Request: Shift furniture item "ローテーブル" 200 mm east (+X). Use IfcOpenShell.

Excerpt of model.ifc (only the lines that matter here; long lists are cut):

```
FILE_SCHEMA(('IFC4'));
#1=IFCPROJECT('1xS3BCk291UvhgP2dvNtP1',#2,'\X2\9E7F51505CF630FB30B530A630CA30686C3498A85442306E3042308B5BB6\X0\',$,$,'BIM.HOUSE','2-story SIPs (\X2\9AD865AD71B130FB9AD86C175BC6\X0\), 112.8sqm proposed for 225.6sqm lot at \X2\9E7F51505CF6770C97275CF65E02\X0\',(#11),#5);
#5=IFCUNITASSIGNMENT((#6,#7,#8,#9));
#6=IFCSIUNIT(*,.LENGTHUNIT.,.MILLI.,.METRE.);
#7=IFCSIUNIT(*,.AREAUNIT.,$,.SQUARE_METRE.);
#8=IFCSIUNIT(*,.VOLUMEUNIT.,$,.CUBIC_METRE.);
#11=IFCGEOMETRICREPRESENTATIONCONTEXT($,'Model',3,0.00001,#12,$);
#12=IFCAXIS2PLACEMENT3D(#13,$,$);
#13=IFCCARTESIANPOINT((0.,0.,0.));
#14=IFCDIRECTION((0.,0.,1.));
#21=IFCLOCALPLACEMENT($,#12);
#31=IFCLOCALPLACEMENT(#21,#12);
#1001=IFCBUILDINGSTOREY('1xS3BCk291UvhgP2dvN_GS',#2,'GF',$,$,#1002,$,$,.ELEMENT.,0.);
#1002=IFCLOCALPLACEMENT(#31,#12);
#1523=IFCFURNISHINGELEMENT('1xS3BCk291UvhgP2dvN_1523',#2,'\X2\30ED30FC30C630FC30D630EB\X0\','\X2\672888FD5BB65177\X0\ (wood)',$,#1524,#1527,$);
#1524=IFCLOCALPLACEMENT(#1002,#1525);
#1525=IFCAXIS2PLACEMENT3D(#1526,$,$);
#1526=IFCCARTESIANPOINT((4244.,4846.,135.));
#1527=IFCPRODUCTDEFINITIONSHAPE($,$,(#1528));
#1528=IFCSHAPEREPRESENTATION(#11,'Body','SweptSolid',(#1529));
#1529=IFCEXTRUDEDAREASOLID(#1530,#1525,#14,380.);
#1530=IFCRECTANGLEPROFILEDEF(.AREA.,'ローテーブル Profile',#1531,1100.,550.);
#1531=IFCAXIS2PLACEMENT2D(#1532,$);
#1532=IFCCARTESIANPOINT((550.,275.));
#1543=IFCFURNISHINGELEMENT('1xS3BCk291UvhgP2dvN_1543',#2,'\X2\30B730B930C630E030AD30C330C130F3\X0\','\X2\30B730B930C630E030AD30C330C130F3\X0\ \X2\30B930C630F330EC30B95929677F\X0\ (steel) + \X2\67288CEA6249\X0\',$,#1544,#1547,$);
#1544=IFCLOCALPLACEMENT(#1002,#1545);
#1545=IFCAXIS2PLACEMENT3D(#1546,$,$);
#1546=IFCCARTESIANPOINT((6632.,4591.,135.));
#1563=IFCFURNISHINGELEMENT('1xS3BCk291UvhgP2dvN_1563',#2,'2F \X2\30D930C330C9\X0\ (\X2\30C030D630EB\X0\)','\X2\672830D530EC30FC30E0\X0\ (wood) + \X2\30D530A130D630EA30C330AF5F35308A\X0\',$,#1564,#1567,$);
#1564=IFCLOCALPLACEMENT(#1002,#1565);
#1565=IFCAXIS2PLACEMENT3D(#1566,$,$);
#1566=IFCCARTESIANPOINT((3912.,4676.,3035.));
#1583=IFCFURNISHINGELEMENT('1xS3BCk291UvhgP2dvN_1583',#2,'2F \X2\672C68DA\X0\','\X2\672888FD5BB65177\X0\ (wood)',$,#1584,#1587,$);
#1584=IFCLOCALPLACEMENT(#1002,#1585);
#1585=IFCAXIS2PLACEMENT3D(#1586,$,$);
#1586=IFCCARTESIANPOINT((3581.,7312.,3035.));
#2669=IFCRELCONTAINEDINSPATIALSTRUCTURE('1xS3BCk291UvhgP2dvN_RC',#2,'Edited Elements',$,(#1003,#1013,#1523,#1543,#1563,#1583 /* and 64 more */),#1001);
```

```python
import ifcopenshell
import ifcopenshell.api.geometry
import ifcopenshell.util.placement
import ifcopenshell.util.unit

model = ifcopenshell.open("model.ifc")
unit_scale = ifcopenshell.util.unit.calculate_unit_scale(model)

item = model.by_guid("1xS3BCk291UvhgP2dvN_1523")
matrix = ifcopenshell.util.placement.get_local_placement(item.ObjectPlacement)
matrix[0, 3] += 0.2 / unit_scale
ifcopenshell.api.geometry.edit_object_placement(model, product=item, matrix=matrix, is_si=False)

print(ifcopenshell.util.placement.get_local_placement(item.ObjectPlacement).round(3) + 0.0)

model.write("model_v2.ifc")
```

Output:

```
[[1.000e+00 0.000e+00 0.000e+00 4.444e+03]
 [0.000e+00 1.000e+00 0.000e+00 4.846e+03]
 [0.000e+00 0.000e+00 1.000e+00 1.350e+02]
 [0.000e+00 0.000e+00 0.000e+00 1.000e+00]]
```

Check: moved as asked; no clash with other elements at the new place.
